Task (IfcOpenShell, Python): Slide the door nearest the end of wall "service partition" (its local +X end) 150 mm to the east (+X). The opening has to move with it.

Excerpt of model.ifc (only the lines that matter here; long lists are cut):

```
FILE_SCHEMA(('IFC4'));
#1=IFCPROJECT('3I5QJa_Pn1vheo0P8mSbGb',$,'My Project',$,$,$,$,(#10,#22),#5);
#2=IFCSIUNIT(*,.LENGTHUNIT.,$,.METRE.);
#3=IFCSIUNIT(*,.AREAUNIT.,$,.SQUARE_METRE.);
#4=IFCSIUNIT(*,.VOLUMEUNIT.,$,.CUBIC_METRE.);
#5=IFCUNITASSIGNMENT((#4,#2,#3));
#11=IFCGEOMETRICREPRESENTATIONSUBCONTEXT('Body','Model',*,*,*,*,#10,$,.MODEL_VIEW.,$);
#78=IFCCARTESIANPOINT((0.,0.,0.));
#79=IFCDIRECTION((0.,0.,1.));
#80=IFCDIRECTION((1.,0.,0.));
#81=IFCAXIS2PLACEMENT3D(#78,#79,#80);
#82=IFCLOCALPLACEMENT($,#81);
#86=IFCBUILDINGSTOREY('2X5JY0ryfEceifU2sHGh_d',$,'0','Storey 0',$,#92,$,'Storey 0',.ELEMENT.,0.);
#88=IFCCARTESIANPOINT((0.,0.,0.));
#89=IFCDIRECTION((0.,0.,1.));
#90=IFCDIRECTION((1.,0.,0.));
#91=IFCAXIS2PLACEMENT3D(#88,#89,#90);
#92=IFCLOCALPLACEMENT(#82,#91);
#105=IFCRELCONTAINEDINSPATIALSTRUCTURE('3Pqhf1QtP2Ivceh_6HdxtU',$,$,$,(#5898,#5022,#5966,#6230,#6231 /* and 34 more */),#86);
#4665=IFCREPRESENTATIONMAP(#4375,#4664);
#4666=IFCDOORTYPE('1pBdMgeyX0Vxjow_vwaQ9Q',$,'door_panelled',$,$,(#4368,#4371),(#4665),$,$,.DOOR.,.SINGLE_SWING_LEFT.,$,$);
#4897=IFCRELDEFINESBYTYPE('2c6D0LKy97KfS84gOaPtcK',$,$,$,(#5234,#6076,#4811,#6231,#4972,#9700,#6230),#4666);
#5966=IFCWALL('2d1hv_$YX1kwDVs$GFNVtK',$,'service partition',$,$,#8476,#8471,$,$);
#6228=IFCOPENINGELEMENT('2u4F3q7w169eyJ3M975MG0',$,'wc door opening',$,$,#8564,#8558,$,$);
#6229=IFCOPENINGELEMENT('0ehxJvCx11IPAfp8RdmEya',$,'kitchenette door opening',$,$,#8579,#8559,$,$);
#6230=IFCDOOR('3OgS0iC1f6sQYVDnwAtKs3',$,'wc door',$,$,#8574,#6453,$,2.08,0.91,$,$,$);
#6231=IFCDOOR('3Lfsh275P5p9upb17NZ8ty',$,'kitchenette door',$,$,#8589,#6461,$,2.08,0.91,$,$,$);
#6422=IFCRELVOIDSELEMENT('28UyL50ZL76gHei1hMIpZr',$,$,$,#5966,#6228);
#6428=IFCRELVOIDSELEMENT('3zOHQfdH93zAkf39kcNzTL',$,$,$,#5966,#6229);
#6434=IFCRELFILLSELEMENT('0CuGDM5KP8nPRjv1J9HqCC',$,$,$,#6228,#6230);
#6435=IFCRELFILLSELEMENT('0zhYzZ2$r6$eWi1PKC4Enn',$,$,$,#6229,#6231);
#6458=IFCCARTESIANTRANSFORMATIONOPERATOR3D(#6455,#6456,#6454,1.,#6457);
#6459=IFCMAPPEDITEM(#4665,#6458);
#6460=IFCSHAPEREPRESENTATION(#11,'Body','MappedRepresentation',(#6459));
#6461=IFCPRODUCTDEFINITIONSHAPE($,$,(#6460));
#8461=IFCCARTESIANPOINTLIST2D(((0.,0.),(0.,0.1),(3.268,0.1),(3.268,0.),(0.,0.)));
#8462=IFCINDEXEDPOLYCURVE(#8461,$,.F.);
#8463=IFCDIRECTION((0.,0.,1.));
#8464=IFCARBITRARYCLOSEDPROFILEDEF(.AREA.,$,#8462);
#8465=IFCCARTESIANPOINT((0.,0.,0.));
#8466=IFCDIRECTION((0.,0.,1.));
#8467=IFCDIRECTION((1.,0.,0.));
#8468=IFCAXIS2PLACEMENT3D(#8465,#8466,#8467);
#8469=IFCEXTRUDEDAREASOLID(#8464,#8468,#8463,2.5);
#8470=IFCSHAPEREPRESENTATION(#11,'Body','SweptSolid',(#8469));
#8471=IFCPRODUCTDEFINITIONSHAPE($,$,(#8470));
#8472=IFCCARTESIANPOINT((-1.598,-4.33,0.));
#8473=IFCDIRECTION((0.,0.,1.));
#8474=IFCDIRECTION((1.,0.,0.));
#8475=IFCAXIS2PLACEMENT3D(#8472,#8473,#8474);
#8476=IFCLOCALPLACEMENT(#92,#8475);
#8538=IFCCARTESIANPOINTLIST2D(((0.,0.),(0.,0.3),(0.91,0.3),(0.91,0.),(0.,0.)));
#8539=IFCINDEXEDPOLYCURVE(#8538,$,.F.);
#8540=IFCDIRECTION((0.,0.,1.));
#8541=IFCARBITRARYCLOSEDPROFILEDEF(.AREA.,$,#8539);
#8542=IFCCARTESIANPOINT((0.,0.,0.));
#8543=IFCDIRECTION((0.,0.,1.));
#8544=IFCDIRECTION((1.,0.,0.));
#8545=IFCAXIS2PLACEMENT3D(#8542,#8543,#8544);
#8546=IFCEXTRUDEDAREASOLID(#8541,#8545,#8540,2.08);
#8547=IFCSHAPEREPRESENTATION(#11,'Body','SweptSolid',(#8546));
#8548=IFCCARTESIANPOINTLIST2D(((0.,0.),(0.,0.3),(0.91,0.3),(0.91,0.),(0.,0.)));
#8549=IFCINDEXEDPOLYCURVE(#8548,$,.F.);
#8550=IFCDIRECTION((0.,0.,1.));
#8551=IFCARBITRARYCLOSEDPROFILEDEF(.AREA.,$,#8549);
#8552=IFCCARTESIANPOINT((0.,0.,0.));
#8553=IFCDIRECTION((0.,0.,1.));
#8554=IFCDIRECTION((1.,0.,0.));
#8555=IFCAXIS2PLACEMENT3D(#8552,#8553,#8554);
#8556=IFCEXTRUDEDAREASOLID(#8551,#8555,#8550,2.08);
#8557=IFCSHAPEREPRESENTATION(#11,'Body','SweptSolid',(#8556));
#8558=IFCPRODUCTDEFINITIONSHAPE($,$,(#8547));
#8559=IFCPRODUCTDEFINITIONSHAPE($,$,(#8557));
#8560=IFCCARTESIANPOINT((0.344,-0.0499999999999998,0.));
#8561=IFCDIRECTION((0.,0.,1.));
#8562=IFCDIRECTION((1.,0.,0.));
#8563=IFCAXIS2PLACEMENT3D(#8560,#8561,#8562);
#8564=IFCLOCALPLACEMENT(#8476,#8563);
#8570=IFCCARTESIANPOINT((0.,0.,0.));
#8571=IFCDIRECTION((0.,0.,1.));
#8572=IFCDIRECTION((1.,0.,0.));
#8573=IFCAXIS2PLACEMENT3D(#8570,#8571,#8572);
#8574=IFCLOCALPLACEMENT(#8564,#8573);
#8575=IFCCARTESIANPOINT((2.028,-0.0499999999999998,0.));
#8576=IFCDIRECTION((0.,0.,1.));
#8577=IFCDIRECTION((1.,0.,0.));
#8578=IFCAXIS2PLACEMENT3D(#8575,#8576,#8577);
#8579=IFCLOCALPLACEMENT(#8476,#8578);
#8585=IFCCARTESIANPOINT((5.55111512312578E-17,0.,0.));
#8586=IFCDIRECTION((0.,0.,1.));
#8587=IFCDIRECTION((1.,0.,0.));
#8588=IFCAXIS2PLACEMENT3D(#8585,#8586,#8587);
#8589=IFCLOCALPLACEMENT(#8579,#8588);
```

```python
import ifcopenshell
import ifcopenshell.api.geometry
import ifcopenshell.util.placement
import ifcopenshell.util.unit

model = ifcopenshell.open("model.ifc")
unit_scale = ifcopenshell.util.unit.calculate_unit_scale(model)

door = model.by_id(6231)
opening = door.FillsVoids[0].RelatingOpeningElement
wall = opening.VoidsElements[0].RelatingBuildingElement

wall_matrix = ifcopenshell.util.placement.get_local_placement(wall.ObjectPlacement)
shift = wall_matrix[:3, 0] * 0.15 / unit_scale
before = ifcopenshell.util.placement.get_local_placement(door.ObjectPlacement)[:3, 3].copy()

# The door is placed relative to its opening, so it follows when the opening moves.
matrix = ifcopenshell.util.placement.get_local_placement(opening.ObjectPlacement)
matrix[:3, 3] += shift
ifcopenshell.api.geometry.edit_object_placement(
    model, product=opening, matrix=matrix, is_si=False, should_transform_children=True
)

after = ifcopenshell.util.placement.get_local_placement(door.ObjectPlacement)[:3, 3]
print("door moved by", (after - before).round(3) + 0.0)

model.write("model_rev.ifc")
```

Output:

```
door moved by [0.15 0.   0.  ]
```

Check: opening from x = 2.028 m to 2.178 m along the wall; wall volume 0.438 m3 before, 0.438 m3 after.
